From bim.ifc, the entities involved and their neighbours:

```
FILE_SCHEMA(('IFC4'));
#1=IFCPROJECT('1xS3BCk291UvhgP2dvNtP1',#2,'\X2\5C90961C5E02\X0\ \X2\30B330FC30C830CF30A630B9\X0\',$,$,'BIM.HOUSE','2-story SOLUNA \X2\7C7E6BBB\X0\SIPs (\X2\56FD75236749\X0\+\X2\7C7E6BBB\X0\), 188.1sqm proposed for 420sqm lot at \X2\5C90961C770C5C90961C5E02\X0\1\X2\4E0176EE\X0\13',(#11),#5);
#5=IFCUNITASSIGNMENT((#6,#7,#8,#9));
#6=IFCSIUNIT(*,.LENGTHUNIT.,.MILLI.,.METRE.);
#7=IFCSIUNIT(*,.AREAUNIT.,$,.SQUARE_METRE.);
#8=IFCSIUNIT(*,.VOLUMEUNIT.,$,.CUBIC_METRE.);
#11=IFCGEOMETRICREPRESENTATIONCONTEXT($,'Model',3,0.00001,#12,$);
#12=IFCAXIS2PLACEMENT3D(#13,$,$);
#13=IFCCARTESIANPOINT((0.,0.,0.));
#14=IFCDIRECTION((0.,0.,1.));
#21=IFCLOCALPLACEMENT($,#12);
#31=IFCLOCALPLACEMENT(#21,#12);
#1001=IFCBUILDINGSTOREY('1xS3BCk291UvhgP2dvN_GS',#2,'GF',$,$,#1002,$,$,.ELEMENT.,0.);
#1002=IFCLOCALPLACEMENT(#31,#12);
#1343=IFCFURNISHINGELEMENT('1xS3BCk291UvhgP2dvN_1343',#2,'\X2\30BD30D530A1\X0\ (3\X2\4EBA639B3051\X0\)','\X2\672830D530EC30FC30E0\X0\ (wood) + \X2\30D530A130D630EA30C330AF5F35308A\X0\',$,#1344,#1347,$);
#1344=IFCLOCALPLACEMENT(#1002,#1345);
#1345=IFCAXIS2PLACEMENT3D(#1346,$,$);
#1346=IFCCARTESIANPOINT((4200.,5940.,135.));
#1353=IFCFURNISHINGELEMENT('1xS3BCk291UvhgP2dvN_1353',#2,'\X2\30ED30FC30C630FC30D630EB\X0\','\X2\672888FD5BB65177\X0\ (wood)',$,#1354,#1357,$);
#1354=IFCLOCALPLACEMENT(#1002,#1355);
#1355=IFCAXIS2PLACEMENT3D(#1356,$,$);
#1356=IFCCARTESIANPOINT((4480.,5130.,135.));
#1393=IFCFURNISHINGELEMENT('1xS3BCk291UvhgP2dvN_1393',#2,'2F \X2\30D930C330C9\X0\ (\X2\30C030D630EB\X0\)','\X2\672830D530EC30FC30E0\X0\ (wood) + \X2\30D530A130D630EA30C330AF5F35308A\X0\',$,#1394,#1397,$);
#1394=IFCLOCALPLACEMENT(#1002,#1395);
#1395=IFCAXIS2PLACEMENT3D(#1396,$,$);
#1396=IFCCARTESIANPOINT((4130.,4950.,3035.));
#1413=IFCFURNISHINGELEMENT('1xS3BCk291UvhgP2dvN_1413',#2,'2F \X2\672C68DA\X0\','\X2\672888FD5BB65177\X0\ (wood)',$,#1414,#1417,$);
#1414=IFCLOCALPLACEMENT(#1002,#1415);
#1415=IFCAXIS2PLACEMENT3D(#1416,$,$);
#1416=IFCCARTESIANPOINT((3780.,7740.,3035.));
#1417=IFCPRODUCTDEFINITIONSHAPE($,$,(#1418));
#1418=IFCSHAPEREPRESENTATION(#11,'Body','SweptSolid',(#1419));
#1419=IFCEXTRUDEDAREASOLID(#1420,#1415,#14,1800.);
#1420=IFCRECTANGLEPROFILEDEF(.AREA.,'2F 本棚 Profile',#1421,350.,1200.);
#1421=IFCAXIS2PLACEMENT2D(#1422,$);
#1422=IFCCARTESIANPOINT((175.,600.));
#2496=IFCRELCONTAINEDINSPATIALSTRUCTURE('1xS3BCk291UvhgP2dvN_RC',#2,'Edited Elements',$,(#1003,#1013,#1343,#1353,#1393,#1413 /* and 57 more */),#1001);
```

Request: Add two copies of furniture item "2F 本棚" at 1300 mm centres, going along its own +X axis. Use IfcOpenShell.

```python
import ifcopenshell
import ifcopenshell.api.geometry
import ifcopenshell.api.root
import ifcopenshell.util.element
import ifcopenshell.util.placement
import ifcopenshell.util.unit

model = ifcopenshell.open("bim.ifc")
unit_scale = ifcopenshell.util.unit.calculate_unit_scale(model)


def reuse_history(source, copy):
    """copy_class also copies each property set's owner history, people and application; keep the originals."""
    for rel in copy.IsDefinedBy:
        if rel.is_a("IfcRelDefinesByProperties") and (history := rel.RelatingPropertyDefinition.OwnerHistory):
            rel.RelatingPropertyDefinition.OwnerHistory = source.OwnerHistory
            ifcopenshell.util.element.remove_deep2(model, history)


source = model.by_id(1413)
base = ifcopenshell.util.placement.get_local_placement(source.ObjectPlacement)
step = base[:3, 0] * 1.3 / unit_scale

for i in range(1, 3):
    copy = ifcopenshell.api.root.copy_class(model, product=source)
    copy.Representation = ifcopenshell.util.element.copy_deep(
        model, source.Representation, exclude=["IfcGeometricRepresentationContext", "IfcRepresentationMap"]
    )
    reuse_history(source, copy)
    matrix = base.copy()
    matrix[:3, 3] += i * step
    print("added at", matrix[:3, 3].round(3) + 0.0)
    ifcopenshell.api.geometry.edit_object_placement(model, product=copy, matrix=matrix, is_si=False)

model.write("bim_v2.ifc")
```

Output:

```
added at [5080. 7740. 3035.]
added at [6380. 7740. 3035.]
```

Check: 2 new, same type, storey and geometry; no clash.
